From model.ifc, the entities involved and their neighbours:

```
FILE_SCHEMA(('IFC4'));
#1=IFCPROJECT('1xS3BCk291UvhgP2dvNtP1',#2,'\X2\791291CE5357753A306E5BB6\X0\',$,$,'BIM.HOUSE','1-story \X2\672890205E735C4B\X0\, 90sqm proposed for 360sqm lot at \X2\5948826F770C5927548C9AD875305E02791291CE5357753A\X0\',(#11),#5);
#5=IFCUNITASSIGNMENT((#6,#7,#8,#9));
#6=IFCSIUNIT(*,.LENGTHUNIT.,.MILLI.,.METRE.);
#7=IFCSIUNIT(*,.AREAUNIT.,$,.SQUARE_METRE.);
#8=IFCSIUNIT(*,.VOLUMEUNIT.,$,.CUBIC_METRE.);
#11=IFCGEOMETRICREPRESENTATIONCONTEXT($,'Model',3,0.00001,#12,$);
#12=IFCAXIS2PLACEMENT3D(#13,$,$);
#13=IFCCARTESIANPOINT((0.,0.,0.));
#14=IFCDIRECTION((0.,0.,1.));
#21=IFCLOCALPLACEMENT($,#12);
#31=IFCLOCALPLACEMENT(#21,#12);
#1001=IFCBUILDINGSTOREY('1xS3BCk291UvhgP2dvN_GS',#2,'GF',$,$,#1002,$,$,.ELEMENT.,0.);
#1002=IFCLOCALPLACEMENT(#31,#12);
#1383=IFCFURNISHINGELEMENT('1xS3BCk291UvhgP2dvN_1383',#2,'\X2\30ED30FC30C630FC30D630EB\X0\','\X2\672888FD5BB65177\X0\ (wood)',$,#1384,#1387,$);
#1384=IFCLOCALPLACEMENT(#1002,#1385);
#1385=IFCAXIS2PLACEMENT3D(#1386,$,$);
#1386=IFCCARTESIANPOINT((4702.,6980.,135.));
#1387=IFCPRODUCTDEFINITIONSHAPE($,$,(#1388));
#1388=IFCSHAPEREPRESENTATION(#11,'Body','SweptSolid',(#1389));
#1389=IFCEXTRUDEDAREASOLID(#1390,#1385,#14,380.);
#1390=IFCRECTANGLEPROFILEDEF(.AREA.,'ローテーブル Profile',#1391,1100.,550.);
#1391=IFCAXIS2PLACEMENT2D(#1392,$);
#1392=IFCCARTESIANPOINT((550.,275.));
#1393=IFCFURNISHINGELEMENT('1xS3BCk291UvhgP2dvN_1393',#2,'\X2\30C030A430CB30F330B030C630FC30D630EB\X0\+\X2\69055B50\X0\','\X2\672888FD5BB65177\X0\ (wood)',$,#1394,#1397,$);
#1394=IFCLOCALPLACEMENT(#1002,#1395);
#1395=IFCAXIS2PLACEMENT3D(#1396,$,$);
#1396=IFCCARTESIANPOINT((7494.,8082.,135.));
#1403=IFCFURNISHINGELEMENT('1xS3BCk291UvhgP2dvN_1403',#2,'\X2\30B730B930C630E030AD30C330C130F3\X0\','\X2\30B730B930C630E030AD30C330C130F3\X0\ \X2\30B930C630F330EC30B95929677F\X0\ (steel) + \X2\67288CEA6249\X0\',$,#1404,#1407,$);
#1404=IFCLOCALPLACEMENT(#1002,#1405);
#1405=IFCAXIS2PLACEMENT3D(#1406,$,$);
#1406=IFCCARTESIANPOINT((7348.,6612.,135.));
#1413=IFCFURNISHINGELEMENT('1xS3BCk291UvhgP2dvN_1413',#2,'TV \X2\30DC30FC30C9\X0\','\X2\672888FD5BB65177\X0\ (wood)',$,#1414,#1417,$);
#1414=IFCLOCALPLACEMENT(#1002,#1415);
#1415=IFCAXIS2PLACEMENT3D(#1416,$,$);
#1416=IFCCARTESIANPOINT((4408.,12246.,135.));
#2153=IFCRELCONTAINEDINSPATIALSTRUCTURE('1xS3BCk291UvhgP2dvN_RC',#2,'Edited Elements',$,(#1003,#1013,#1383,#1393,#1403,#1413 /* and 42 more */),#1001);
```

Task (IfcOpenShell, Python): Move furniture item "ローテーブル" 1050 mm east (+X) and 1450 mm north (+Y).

```python
import ifcopenshell
import ifcopenshell.api.geometry
import ifcopenshell.util.placement
import ifcopenshell.util.unit

model = ifcopenshell.open("model.ifc")
unit_scale = ifcopenshell.util.unit.calculate_unit_scale(model)

item = model.by_guid("1xS3BCk291UvhgP2dvN_1383")
matrix = ifcopenshell.util.placement.get_local_placement(item.ObjectPlacement)
matrix[0, 3] += 1.05 / unit_scale
matrix[1, 3] += 1.45 / unit_scale
ifcopenshell.api.geometry.edit_object_placement(model, product=item, matrix=matrix, is_si=False)

print(ifcopenshell.util.placement.get_local_placement(item.ObjectPlacement).round(3) + 0.0)

model.write("model_edited.ifc")
```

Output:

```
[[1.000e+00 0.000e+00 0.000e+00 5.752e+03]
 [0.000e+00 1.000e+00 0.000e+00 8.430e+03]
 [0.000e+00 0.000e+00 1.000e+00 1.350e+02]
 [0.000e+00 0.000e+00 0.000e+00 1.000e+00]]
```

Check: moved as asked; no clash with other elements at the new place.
